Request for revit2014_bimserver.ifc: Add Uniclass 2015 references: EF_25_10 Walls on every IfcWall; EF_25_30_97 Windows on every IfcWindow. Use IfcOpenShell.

First a look at what the model holds.

```python
import ifcopenshell

model = ifcopenshell.open("revit2014_bimserver.ifc")
print(model.schema)
print("classifications:", [c.Name for c in model.by_type("IfcClassification")])
for ifc_class in ("IfcDoor", "IfcRoof", "IfcStair", "IfcWall", "IfcWindow"):
    print(ifc_class, len(model.by_type(ifc_class)))
```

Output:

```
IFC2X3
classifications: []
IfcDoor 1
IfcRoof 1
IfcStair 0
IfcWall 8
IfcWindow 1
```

```python
import ifcopenshell
import ifcopenshell.api.classification

model = ifcopenshell.open("revit2014_bimserver.ifc")

# IFC2X3 requires Source and Edition and has no link from the project to the system.
system = model.create_entity("IfcClassification", Source="NBS", Edition="2015", Name="Uniclass 2015")

codes = {
    "IfcWall": ("EF_25_10", "Walls"),
    "IfcWindow": ("EF_25_30_97", "Windows"),
}
for ifc_class, (code, name) in codes.items():
    products = model.by_type(ifc_class)
    ifcopenshell.api.classification.add_reference(
        model, products=products, classification=system, identification=code, name=name
    )
    print(code, len(products))

model.write("revit2014_bimserver_edited.ifc")
```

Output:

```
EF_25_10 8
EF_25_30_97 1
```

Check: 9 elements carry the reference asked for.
